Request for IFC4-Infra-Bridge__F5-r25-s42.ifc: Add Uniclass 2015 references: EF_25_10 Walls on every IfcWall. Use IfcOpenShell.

First a look at what the model holds.

```python
import ifcopenshell

model = ifcopenshell.open("IFC4-Infra-Bridge__F5-r25-s42.ifc")
print(model.schema)
print("classifications:", [c.Name for c in model.by_type("IfcClassification")])
for ifc_class in ("IfcDoor", "IfcRoof", "IfcStair", "IfcWall", "IfcWindow"):
    print(ifc_class, len(model.by_type(ifc_class)))
```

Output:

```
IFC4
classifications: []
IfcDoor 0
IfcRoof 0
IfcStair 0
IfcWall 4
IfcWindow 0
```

```python
import ifcopenshell
import ifcopenshell.api.classification

model = ifcopenshell.open("IFC4-Infra-Bridge__F5-r25-s42.ifc")

system = ifcopenshell.api.classification.add_classification(model, classification="Uniclass 2015")

codes = {
    "IfcWall": ("EF_25_10", "Walls"),
}
for ifc_class, (code, name) in codes.items():
    products = model.by_type(ifc_class)
    ifcopenshell.api.classification.add_reference(
        model, products=products, classification=system, identification=code, name=name
    )
    print(code, len(products))

model.write("IFC4-Infra-Bridge__F5-r25-s42_v2.ifc")
```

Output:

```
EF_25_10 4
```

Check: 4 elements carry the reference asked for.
